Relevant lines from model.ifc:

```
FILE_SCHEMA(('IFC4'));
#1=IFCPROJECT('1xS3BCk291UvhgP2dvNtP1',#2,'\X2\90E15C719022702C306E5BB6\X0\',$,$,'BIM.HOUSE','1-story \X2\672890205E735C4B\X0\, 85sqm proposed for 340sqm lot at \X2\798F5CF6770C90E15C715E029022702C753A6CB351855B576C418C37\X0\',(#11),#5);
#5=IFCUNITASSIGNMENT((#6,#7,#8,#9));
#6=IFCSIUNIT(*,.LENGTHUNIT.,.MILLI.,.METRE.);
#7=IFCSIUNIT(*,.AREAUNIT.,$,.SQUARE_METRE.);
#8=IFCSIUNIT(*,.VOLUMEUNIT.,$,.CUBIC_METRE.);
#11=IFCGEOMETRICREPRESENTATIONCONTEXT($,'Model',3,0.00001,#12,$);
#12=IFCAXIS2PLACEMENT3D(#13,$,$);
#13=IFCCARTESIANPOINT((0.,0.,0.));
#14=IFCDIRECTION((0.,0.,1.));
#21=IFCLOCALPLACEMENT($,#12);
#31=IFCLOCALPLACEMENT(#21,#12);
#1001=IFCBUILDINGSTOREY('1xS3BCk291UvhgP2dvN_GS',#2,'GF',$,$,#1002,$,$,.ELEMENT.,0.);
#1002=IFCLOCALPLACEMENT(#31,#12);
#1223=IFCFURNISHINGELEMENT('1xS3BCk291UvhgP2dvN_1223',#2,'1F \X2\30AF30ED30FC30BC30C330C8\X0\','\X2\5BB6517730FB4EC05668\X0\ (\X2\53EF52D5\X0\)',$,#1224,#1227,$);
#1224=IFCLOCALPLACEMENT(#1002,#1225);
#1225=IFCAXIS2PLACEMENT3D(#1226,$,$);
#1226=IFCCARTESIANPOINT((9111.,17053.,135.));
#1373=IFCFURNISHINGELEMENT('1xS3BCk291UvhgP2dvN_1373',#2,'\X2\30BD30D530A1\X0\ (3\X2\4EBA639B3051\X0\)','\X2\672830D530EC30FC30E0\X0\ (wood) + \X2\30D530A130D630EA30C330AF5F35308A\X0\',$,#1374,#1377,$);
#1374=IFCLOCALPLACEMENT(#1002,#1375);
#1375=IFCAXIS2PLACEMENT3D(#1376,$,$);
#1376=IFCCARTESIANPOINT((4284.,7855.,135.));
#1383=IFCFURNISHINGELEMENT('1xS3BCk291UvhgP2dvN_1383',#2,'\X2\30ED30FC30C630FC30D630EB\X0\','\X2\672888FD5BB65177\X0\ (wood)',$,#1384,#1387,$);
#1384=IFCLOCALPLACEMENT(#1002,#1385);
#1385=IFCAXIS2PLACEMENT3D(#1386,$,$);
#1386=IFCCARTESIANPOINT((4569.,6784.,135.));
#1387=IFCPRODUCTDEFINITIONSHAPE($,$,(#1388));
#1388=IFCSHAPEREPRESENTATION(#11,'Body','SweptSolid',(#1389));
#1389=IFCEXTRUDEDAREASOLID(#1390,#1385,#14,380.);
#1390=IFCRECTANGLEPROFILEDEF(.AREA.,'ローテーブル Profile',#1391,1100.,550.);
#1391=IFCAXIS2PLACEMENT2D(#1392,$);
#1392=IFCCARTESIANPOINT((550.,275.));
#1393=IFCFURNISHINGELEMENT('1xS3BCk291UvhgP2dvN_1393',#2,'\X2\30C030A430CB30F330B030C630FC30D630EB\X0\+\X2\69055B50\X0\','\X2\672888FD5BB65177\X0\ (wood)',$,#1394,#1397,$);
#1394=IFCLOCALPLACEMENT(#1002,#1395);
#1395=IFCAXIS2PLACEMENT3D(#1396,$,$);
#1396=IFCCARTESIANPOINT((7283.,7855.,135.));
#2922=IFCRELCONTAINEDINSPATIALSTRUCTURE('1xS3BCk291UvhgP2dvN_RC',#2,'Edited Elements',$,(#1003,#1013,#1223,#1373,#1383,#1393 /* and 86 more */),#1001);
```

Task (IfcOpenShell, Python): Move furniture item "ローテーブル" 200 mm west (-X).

```python
import ifcopenshell
import ifcopenshell.api.geometry
import ifcopenshell.util.placement
import ifcopenshell.util.unit

model = ifcopenshell.open("model.ifc")
unit_scale = ifcopenshell.util.unit.calculate_unit_scale(model)

item = model.by_guid("1xS3BCk291UvhgP2dvN_1383")
matrix = ifcopenshell.util.placement.get_local_placement(item.ObjectPlacement)
matrix[0, 3] -= 0.2 / unit_scale
ifcopenshell.api.geometry.edit_object_placement(model, product=item, matrix=matrix, is_si=False)

print(ifcopenshell.util.placement.get_local_placement(item.ObjectPlacement).round(3) + 0.0)

model.write("model_edited.ifc")
```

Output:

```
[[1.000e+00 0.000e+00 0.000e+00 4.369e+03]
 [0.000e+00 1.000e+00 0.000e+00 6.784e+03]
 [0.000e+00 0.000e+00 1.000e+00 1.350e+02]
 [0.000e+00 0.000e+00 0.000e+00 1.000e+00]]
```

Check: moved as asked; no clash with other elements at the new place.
